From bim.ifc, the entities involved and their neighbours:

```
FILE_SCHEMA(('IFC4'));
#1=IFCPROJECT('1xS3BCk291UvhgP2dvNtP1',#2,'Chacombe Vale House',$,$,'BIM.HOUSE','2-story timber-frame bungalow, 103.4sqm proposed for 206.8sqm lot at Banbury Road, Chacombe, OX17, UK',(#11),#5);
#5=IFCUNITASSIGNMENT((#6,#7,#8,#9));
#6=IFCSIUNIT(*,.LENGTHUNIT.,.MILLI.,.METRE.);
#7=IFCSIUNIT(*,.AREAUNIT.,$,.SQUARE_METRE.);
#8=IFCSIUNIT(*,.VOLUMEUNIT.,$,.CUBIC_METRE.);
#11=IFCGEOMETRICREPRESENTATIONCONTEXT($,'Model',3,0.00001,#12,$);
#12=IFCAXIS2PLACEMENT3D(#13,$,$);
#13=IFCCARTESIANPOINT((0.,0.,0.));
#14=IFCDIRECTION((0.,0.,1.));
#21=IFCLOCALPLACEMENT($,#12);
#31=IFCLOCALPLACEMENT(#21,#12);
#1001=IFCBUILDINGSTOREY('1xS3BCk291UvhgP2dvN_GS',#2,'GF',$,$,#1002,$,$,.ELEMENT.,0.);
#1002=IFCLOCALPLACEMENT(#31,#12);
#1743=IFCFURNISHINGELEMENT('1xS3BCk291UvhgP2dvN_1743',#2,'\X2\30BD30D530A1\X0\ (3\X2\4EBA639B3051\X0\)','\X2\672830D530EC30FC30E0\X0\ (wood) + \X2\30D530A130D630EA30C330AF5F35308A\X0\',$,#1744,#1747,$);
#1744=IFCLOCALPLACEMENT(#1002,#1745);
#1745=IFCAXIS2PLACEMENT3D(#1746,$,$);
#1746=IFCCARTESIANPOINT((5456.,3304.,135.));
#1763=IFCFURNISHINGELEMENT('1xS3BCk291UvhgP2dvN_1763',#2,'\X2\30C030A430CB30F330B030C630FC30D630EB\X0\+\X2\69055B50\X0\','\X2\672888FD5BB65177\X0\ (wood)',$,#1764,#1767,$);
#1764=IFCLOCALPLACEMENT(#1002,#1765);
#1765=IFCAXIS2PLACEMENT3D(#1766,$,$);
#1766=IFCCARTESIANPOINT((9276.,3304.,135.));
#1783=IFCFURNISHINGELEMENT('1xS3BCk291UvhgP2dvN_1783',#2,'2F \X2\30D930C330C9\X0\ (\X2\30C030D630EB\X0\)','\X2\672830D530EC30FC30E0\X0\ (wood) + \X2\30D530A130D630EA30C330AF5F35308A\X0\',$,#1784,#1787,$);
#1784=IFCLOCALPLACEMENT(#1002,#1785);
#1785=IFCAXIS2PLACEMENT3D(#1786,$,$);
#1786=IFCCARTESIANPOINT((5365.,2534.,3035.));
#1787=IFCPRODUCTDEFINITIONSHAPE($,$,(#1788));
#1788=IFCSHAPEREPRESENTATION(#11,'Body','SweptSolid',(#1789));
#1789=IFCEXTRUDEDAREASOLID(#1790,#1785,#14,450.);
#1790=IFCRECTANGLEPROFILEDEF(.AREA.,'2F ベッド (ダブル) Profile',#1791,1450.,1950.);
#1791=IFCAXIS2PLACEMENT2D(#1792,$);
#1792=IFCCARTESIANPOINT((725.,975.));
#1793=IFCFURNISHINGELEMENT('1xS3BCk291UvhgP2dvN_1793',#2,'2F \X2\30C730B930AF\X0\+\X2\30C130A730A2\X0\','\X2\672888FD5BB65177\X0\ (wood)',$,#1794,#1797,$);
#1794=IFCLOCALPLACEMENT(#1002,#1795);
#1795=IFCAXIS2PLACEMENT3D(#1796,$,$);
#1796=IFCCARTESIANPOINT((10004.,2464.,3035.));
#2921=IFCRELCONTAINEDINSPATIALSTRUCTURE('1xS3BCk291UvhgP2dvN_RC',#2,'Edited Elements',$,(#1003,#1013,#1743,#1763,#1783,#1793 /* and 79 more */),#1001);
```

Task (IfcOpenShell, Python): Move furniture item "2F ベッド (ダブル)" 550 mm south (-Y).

```python
import ifcopenshell
import ifcopenshell.api.geometry
import ifcopenshell.util.placement

model = ifcopenshell.open("bim.ifc")

item = model.by_id(1783)
matrix = ifcopenshell.util.placement.get_local_placement(item.ObjectPlacement)
matrix[1, 3] -= 550.0
ifcopenshell.api.geometry.edit_object_placement(model, product=item, matrix=matrix, is_si=False)

print(ifcopenshell.util.placement.get_local_placement(item.ObjectPlacement).round(3) + 0.0)

model.write("bim_updated.ifc")
```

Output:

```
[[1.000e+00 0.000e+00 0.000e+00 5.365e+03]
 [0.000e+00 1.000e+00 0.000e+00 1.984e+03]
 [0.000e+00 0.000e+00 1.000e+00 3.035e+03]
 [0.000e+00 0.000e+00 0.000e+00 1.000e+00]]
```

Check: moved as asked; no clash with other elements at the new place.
